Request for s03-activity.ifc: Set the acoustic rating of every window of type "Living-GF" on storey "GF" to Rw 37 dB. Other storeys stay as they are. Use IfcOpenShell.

First a look at what the model holds.

```python
import ifcopenshell
import ifcopenshell.util.element

model = ifcopenshell.open("s03-activity.ifc")
print(model.schema)
storey = next(s for s in model.by_type("IfcBuildingStorey") if s.Name == "GF")
windows = [e for e in ifcopenshell.util.element.get_decomposition(storey) if e.is_a("IfcWindow")]
seen = {}
for e in windows:
    element_type = ifcopenshell.util.element.get_type(e)
    key = (element_type.Name if element_type != e and element_type else None, ifcopenshell.util.element.get_pset(e, "Pset_WindowCommon", "AcousticRating"))
    seen[key] = seen.get(key, 0) + 1
for (name, value), count in sorted(seen.items(), key=str):
    print(count, "x", name, "|", value)
```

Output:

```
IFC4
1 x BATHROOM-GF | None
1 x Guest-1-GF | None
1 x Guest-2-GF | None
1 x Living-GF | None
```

```python
import ifcopenshell
import ifcopenshell.api.pset
import ifcopenshell.util.element

model = ifcopenshell.open("s03-activity.ifc")

storey = next(s for s in model.by_type("IfcBuildingStorey") if s.Name == "GF")
windows = [e for e in ifcopenshell.util.element.get_decomposition(storey) if e.is_a("IfcWindow")]

count = 0
for e in windows:
    element_type = ifcopenshell.util.element.get_type(e)
    if element_type in (None, e) or element_type.Name != "Living-GF":
        continue
    # add_pset returns the element's existing set when there is one.
    pset = ifcopenshell.api.pset.add_pset(model, product=e, name="Pset_WindowCommon")
    ifcopenshell.api.pset.edit_pset(model, pset=pset, properties={"AcousticRating": "Rw 37 dB"})
    count += 1

print(count, "windows updated")

model.write("s03-activity_updated.ifc")
```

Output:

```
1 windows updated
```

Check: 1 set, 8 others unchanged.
